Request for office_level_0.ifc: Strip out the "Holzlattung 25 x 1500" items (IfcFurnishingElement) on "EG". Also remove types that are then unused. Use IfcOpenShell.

First a look at what the model holds.

```python
import ifcopenshell
import ifcopenshell.util.element

model = ifcopenshell.open("office_level_0.ifc")
print(model.schema)
storey = next(s for s in model.by_type("IfcBuildingStorey") if s.Name == "EG")
furniture = [e for e in ifcopenshell.util.element.get_decomposition(storey) if e.is_a("IfcFurnishingElement")]
seen = {}
for e in furniture:
    element_type = ifcopenshell.util.element.get_type(e)
    name = element_type.Name if element_type not in (None, e) else None
    seen[name] = seen.get(name, 0) + 1
for name, count in sorted(seen.items(), key=str):
    print(count, "x", name)
```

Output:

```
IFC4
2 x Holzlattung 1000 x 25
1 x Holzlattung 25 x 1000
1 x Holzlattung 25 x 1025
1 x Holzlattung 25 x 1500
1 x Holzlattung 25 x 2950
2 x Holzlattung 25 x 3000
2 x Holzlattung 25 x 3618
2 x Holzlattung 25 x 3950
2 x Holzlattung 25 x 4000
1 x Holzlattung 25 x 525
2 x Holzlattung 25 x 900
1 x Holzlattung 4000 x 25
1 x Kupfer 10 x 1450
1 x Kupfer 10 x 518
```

```python
import ifcopenshell
import ifcopenshell.api.root
import ifcopenshell.util.element

model = ifcopenshell.open("office_level_0.ifc")

storey = next(s for s in model.by_type("IfcBuildingStorey") if s.Name == "EG")
furniture = [e for e in ifcopenshell.util.element.get_decomposition(storey) if e.is_a("IfcFurnishingElement")]
targets = [e for e in furniture if (t := ifcopenshell.util.element.get_type(e)) not in (None, e) and t.Name == "Holzlattung 25 x 1500"]
types = {ifcopenshell.util.element.get_type(e) for e in targets} - {None, *targets}

for e in targets:
    ifcopenshell.api.root.remove_product(model, product=e)
print(len(targets), "removed")

unused = [t for t in types if not ifcopenshell.util.element.get_types(t)]
for t in unused:
    ifcopenshell.api.root.remove_product(model, product=t)
print(len(unused), "unused types removed")

model.write("office_level_0_updated.ifc")
```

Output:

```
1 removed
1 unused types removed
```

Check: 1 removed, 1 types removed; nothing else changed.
